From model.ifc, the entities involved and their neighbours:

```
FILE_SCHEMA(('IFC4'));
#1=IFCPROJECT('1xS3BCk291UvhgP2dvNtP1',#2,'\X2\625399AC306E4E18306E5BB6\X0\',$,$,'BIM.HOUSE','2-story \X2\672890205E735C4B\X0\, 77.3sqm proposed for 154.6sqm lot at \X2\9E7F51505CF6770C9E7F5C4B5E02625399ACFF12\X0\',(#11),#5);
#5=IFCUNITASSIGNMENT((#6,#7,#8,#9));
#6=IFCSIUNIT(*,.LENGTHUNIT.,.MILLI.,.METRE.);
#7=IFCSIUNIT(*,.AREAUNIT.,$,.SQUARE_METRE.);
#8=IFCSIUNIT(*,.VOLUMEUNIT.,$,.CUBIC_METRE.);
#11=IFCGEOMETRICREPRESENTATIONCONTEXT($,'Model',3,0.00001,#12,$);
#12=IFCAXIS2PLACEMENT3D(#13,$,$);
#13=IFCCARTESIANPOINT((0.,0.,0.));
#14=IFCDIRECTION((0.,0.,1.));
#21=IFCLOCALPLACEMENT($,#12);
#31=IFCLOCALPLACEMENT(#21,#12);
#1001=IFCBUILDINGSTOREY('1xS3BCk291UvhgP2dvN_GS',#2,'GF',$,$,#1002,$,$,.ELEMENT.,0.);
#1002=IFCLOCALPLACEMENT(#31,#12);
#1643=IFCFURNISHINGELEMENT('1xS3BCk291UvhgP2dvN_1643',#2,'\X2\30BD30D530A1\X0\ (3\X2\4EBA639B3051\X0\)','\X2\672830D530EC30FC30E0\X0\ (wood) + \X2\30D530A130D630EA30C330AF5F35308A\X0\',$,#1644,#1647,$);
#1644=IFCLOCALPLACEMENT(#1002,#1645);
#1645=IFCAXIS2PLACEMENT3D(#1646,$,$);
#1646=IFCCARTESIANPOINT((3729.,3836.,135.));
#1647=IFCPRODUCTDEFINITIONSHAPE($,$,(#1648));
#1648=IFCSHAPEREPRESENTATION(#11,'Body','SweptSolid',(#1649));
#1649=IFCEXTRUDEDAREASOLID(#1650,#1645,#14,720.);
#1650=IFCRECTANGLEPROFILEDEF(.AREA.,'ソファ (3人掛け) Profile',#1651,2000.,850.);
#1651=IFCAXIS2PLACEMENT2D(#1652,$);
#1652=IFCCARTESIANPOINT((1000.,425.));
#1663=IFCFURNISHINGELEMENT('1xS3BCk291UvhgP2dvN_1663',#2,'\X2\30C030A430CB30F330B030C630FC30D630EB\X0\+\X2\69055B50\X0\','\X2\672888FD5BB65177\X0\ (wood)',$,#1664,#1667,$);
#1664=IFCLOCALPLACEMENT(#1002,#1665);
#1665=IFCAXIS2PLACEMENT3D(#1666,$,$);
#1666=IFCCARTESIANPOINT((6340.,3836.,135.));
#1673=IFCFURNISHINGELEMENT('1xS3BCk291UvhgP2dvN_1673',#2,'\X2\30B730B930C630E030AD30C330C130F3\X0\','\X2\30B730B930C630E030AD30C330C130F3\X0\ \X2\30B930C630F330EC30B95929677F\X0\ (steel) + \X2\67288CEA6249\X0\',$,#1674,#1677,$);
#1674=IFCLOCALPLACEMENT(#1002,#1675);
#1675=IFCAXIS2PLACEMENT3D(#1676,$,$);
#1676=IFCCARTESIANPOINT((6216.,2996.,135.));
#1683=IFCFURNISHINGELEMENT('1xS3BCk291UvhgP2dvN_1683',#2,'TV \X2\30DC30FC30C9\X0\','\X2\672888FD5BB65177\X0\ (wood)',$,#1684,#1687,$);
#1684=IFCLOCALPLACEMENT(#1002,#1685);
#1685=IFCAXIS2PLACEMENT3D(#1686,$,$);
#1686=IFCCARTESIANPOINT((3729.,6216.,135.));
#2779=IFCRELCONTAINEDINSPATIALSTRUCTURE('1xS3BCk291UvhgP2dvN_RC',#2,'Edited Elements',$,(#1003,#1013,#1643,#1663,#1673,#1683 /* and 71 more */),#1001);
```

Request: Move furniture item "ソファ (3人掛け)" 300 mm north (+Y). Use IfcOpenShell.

```python
import ifcopenshell
import ifcopenshell.api.geometry
import ifcopenshell.util.placement
import ifcopenshell.util.unit

model = ifcopenshell.open("model.ifc")
unit_scale = ifcopenshell.util.unit.calculate_unit_scale(model)

item = model.by_guid("1xS3BCk291UvhgP2dvN_1643")
matrix = ifcopenshell.util.placement.get_local_placement(item.ObjectPlacement)
matrix[1, 3] += 0.3 / unit_scale
ifcopenshell.api.geometry.edit_object_placement(model, product=item, matrix=matrix, is_si=False)

print(ifcopenshell.util.placement.get_local_placement(item.ObjectPlacement).round(3) + 0.0)

model.write("model_updated.ifc")
```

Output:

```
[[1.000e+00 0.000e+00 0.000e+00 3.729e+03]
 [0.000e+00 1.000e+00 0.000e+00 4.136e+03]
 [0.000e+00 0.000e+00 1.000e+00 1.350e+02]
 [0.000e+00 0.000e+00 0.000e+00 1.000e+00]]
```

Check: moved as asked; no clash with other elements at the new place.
